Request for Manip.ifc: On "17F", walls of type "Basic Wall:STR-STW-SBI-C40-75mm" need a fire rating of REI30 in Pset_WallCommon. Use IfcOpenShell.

First a look at what the model holds.

```python
import ifcopenshell
import ifcopenshell.util.element

model = ifcopenshell.open("Manip.ifc")
print(model.schema)
storey = next(s for s in model.by_type("IfcBuildingStorey") if s.Name == "17F")
walls = [e for e in ifcopenshell.util.element.get_decomposition(storey) if e.is_a("IfcWall")]
seen = {}
for e in walls:
    element_type = ifcopenshell.util.element.get_type(e)
    key = (element_type.Name if element_type != e and element_type else None, ifcopenshell.util.element.get_pset(e, "Pset_WallCommon", "FireRating"))
    seen[key] = seen.get(key, 0) + 1
for (name, value), count in sorted(seen.items(), key=str):
    print(count, "x", name, "|", value)
```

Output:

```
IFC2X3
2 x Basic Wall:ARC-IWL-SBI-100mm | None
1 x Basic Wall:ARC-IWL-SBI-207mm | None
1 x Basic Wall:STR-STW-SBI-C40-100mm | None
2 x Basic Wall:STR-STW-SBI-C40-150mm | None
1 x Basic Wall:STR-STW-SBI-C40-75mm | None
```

```python
import ifcopenshell
import ifcopenshell.api.pset
import ifcopenshell.util.element

model = ifcopenshell.open("Manip.ifc")

storey = next(s for s in model.by_type("IfcBuildingStorey") if s.Name == "17F")
walls = [e for e in ifcopenshell.util.element.get_decomposition(storey) if e.is_a("IfcWall")]

count = 0
for e in walls:
    element_type = ifcopenshell.util.element.get_type(e)
    if element_type in (None, e) or element_type.Name != "Basic Wall:STR-STW-SBI-C40-75mm":
        continue
    # add_pset returns the element's existing set when there is one.
    pset = ifcopenshell.api.pset.add_pset(model, product=e, name="Pset_WallCommon")
    ifcopenshell.api.pset.edit_pset(model, pset=pset, properties={"FireRating": "REI30"})
    count += 1

print(count, "walls updated")

model.write("Manip-out.ifc")
```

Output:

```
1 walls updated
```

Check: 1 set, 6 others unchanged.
